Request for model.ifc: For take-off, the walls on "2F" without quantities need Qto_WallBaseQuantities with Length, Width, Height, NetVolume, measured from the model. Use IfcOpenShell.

First a look at what the model holds.

```python
import ifcopenshell
import ifcopenshell.util.element
import ifcopenshell.util.unit

model = ifcopenshell.open("model.ifc")
print(model.schema)
for unit_type in ("LENGTHUNIT", "AREAUNIT", "VOLUMEUNIT"):
    print(unit_type, ifcopenshell.util.unit.calculate_unit_scale(model, unit_type))
storey = next(s for s in model.by_type("IfcBuildingStorey") if s.Name == "2F")
walls = [e for e in ifcopenshell.util.element.get_decomposition(storey) if e.is_a("IfcWall")]
for e in sorted(walls, key=lambda e: e.id()):
    print(e.id(), e.is_a(), e.Name, list(ifcopenshell.util.element.get_psets(e, qtos_only=True)), sep=" | ")
```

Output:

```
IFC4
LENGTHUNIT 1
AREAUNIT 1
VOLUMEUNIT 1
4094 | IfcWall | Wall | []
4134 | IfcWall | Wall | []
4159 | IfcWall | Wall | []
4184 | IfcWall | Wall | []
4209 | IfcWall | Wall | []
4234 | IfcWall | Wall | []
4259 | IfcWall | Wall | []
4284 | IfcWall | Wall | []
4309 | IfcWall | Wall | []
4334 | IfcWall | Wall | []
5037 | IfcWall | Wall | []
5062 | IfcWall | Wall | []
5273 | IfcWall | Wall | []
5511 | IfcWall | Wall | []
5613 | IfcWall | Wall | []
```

```python
import ifcopenshell
import ifcopenshell.api.pset
import ifcopenshell.geom
import ifcopenshell.util.element
import ifcopenshell.util.shape
import ifcopenshell.util.unit

model = ifcopenshell.open("model.ifc")
unit_scale = ifcopenshell.util.unit.calculate_unit_scale(model)
volume_scale = ifcopenshell.util.unit.calculate_unit_scale(model, "VOLUMEUNIT")
settings = ifcopenshell.geom.settings()

storey = next(s for s in model.by_type("IfcBuildingStorey") if s.Name == "2F")
walls = [e for e in ifcopenshell.util.element.get_decomposition(storey) if e.is_a("IfcWall")]

for e in sorted(walls, key=lambda e: e.id()):
    if ifcopenshell.util.element.get_psets(e, qtos_only=True, should_inherit=False):
        continue
    # Geometry comes back in metres, in the element's own axes.
    shape = ifcopenshell.geom.create_shape(settings, e)
    values = {
        "Length": ifcopenshell.util.shape.get_x(shape.geometry) / unit_scale,
        "Width": ifcopenshell.util.shape.get_y(shape.geometry) / unit_scale,
        "Height": ifcopenshell.util.shape.get_z(shape.geometry) / unit_scale,
        "NetVolume": ifcopenshell.util.shape.get_volume(shape.geometry) / volume_scale,
    }
    qto = ifcopenshell.api.pset.add_qto(model, product=e, name="Qto_WallBaseQuantities")
    ifcopenshell.api.pset.edit_qto(model, qto=qto, properties=values)
    print(e.id(), {k: round(v, 3) for k, v in values.items()})

model.write("model-out.ifc")
```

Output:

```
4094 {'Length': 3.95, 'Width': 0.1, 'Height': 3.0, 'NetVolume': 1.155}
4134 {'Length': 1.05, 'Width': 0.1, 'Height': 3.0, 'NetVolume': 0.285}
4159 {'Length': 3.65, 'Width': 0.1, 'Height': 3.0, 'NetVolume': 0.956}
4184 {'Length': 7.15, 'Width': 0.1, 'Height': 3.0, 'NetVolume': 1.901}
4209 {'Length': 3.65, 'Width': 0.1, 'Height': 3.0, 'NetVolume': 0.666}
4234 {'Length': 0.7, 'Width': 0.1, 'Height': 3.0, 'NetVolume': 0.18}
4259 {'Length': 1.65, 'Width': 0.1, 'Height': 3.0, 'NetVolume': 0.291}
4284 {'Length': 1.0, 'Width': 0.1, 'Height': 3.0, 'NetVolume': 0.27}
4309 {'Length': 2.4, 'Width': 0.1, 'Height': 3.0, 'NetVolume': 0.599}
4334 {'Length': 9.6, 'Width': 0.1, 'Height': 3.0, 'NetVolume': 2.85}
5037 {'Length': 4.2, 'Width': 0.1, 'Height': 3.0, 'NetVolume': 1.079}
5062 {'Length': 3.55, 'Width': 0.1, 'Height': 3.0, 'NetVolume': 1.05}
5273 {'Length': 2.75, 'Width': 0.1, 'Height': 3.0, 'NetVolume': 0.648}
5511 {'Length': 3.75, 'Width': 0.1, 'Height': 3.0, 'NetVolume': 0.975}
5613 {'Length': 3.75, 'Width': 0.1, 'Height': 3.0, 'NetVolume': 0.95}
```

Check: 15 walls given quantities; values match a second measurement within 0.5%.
